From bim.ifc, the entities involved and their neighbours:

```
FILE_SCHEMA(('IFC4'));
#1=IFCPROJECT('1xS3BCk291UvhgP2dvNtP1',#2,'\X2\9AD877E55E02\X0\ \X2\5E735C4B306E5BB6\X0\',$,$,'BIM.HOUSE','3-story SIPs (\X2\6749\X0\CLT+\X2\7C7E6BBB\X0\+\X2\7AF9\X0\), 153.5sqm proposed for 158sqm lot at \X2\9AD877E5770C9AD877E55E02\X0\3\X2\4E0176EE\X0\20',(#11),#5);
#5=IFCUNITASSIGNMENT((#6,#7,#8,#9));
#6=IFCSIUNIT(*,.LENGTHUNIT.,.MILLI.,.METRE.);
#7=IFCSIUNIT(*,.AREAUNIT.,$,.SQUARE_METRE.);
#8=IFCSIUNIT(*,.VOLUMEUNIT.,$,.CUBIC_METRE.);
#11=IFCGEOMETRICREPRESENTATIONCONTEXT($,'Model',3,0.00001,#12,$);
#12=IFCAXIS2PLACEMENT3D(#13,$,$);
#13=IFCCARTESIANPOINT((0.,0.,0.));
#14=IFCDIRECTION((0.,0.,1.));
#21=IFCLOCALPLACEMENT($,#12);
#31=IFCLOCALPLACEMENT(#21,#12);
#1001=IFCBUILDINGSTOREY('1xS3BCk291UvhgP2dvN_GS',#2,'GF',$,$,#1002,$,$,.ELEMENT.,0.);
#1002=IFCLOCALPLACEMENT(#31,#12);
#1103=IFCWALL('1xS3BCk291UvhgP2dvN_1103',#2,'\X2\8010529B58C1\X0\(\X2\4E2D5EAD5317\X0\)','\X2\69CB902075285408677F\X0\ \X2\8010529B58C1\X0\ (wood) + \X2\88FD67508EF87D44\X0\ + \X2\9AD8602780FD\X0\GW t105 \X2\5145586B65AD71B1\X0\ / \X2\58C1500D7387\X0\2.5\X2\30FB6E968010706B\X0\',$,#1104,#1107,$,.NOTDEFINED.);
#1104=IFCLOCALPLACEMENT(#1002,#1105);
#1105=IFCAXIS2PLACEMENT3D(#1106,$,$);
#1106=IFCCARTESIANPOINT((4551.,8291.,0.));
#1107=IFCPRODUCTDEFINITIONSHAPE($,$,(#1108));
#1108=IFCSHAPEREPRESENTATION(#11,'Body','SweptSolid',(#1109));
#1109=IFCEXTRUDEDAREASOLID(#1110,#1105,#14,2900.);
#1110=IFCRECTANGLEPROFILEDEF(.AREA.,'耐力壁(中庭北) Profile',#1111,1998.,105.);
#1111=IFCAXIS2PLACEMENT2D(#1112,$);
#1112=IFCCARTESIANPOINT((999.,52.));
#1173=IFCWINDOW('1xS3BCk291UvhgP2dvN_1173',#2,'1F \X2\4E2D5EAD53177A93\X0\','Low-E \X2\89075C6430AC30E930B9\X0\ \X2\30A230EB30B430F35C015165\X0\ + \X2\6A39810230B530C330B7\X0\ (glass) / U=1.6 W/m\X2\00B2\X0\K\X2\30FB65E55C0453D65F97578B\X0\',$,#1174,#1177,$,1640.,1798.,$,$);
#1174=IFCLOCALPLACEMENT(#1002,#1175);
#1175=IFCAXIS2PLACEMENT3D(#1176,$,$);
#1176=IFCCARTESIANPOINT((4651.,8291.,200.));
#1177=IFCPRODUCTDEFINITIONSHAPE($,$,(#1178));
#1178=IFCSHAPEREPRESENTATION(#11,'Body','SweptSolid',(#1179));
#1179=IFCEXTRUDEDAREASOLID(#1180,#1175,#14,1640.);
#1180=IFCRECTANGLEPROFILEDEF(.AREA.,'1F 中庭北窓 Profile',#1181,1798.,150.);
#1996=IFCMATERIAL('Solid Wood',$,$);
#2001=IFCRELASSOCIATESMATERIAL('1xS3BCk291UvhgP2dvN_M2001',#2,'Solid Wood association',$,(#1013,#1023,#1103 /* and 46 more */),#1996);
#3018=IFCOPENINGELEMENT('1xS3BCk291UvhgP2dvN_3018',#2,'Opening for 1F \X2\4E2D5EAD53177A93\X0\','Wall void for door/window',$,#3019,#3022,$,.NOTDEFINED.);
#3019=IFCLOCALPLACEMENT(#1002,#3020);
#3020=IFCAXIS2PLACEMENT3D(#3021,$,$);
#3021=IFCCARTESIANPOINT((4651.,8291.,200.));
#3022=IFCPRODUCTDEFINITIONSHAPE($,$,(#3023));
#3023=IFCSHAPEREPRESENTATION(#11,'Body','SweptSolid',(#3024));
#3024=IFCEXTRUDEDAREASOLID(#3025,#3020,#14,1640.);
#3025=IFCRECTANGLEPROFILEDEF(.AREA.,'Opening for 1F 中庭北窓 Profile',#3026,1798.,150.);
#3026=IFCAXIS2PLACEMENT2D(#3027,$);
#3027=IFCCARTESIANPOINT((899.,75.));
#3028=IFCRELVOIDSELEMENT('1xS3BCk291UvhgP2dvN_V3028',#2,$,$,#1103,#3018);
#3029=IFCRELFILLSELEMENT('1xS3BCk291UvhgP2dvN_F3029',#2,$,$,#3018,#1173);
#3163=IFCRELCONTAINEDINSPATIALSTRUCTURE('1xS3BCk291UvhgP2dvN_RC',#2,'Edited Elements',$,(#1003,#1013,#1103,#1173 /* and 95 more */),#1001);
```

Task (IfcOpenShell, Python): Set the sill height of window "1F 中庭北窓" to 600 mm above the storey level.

```python
import numpy as np
import ifcopenshell
import ifcopenshell.api.geometry
import ifcopenshell.geom
import ifcopenshell.util.element
import ifcopenshell.util.placement
import ifcopenshell.util.shape
import ifcopenshell.util.unit

model = ifcopenshell.open("bim.ifc")
unit_scale = ifcopenshell.util.unit.calculate_unit_scale(model)

window = model.by_guid("1xS3BCk291UvhgP2dvN_1173")
opening = window.FillsVoids[0].RelatingOpeningElement
storey = ifcopenshell.util.element.get_container(window, ifc_class="IfcBuildingStorey")
level = ifcopenshell.util.placement.get_local_placement(storey.ObjectPlacement)[2, 3]

# The opening's origin need not be at the sill, so measure its lowest point.
shape = ifcopenshell.geom.create_shape(ifcopenshell.geom.settings(), opening)
bottom = ifcopenshell.util.shape.get_shape_bottom_elevation(shape, shape.geometry) / unit_scale
dz = level + 600.0 - bottom

shift = np.array([0.0, 0.0, dz])
# The window is not placed relative to its opening, so move both.
for product in (opening, window):
    matrix = ifcopenshell.util.placement.get_local_placement(product.ObjectPlacement)
    matrix[:3, 3] += shift
    ifcopenshell.api.geometry.edit_object_placement(model, product=product, matrix=matrix, is_si=False)

print(f"moved by {dz * unit_scale:+.3f} m")

model.write("bim_v2.ifc")
```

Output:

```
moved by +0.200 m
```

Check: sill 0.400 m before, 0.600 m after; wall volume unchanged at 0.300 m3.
